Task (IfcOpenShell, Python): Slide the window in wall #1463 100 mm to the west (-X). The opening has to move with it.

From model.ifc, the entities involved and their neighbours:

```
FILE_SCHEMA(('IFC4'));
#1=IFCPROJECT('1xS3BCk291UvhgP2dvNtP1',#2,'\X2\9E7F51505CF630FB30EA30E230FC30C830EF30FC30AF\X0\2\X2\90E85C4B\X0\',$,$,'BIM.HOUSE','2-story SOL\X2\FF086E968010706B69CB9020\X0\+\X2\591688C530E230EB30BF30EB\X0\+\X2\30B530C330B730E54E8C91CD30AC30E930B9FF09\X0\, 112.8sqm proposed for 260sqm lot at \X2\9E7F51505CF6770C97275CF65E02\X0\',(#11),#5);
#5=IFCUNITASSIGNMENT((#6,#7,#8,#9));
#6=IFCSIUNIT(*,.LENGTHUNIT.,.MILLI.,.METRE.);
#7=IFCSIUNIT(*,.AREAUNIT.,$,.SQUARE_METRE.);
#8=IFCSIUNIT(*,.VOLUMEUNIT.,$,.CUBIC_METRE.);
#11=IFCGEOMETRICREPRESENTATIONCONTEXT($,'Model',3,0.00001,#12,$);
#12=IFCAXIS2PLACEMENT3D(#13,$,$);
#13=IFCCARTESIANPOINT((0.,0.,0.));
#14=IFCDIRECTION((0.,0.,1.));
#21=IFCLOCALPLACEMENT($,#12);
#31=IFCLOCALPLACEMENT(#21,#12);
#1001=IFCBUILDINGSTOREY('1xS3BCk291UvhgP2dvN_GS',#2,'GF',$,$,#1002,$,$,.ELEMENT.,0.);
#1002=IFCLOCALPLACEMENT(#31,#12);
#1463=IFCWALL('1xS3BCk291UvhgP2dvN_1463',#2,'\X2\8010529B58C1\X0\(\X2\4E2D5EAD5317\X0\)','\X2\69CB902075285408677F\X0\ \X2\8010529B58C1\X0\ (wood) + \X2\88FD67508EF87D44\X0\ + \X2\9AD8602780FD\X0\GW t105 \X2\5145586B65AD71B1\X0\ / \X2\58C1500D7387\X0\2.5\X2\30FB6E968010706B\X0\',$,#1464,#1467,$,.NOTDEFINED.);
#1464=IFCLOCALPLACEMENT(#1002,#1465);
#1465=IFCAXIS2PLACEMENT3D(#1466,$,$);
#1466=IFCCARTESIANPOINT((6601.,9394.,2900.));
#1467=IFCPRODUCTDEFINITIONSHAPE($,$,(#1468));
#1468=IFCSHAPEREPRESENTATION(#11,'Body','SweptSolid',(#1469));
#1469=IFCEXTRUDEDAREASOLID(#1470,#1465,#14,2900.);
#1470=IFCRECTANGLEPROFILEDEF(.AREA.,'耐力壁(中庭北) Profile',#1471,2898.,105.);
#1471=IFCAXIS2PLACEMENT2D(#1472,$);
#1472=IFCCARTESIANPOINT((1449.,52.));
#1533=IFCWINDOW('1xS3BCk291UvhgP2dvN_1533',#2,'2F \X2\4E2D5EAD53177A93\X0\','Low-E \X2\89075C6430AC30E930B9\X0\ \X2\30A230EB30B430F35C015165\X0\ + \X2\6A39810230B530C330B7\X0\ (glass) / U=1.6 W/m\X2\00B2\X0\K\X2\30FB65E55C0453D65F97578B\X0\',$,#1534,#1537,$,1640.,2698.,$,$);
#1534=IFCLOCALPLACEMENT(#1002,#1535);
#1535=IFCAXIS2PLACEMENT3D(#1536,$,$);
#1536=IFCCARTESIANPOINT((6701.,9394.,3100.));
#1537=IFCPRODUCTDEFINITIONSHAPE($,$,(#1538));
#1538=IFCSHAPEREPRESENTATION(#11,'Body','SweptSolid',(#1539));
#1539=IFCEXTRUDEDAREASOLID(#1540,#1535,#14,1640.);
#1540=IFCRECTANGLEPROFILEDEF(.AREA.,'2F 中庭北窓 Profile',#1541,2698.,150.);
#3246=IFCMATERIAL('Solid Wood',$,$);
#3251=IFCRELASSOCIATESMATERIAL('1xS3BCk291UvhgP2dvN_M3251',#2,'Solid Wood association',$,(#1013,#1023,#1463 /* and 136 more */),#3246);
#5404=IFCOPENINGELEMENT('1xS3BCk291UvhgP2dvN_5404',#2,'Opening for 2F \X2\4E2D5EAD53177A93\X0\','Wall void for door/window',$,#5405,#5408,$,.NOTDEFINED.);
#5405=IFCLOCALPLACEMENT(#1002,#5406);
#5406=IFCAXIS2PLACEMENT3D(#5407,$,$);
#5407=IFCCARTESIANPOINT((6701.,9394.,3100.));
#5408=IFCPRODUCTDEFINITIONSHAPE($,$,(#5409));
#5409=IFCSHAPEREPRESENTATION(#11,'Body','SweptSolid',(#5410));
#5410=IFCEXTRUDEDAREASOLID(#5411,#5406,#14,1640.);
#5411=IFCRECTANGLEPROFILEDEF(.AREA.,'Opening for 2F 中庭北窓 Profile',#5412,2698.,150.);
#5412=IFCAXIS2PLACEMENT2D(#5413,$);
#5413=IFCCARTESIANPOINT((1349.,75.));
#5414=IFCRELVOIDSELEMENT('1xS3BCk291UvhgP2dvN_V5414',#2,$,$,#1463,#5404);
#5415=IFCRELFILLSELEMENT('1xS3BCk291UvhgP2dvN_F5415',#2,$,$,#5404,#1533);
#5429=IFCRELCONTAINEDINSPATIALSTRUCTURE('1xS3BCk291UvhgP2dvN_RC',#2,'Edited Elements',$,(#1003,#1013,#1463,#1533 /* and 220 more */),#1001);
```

```python
import ifcopenshell
import ifcopenshell.api.geometry
import ifcopenshell.util.placement

model = ifcopenshell.open("model.ifc")

window = model.by_id(1533)
opening = window.FillsVoids[0].RelatingOpeningElement
wall = opening.VoidsElements[0].RelatingBuildingElement

wall_matrix = ifcopenshell.util.placement.get_local_placement(wall.ObjectPlacement)
shift = wall_matrix[:3, 0] * -100.0
before = ifcopenshell.util.placement.get_local_placement(window.ObjectPlacement)[:3, 3].copy()

# The window is not placed relative to its opening, so move both.
for product in (opening, window):
    matrix = ifcopenshell.util.placement.get_local_placement(product.ObjectPlacement)
    matrix[:3, 3] += shift
    ifcopenshell.api.geometry.edit_object_placement(model, product=product, matrix=matrix, is_si=False)

after = ifcopenshell.util.placement.get_local_placement(window.ObjectPlacement)[:3, 3]
print("window moved by", (after - before).round(3) + 0.0)

model.write("model_updated.ifc")
```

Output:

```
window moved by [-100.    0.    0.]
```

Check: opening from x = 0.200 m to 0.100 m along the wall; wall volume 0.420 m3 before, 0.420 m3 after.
